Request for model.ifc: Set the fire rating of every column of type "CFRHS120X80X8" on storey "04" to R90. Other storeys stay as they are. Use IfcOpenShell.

First a look at what the model holds.

```python
import ifcopenshell
import ifcopenshell.util.element

model = ifcopenshell.open("model.ifc")
print(model.schema)
storey = next(s for s in model.by_type("IfcBuildingStorey") if s.Name == "04")
columns = [e for e in ifcopenshell.util.element.get_decomposition(storey) if e.is_a("IfcColumn")]
seen = {}
for e in columns:
    element_type = ifcopenshell.util.element.get_type(e)
    key = (element_type.Name if element_type != e and element_type else None, ifcopenshell.util.element.get_pset(e, "Pset_ColumnCommon", "FireRating"))
    seen[key] = seen.get(key, 0) + 1
for (name, value), count in sorted(seen.items(), key=str):
    print(count, "x", name, "|", value)
```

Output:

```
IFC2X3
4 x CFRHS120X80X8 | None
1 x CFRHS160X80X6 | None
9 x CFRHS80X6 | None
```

```python
import ifcopenshell
import ifcopenshell.api.pset
import ifcopenshell.util.element

model = ifcopenshell.open("model.ifc")

storey = next(s for s in model.by_type("IfcBuildingStorey") if s.Name == "04")
columns = [e for e in ifcopenshell.util.element.get_decomposition(storey) if e.is_a("IfcColumn")]

count = 0
for e in columns:
    element_type = ifcopenshell.util.element.get_type(e)
    if element_type in (None, e) or element_type.Name != "CFRHS120X80X8":
        continue
    # add_pset returns the element's existing set when there is one.
    pset = ifcopenshell.api.pset.add_pset(model, product=e, name="Pset_ColumnCommon")
    ifcopenshell.api.pset.edit_pset(model, pset=pset, properties={"FireRating": "R90"})
    count += 1

print(count, "columns updated")

model.write("model_rev.ifc")
```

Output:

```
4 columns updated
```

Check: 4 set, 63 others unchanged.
